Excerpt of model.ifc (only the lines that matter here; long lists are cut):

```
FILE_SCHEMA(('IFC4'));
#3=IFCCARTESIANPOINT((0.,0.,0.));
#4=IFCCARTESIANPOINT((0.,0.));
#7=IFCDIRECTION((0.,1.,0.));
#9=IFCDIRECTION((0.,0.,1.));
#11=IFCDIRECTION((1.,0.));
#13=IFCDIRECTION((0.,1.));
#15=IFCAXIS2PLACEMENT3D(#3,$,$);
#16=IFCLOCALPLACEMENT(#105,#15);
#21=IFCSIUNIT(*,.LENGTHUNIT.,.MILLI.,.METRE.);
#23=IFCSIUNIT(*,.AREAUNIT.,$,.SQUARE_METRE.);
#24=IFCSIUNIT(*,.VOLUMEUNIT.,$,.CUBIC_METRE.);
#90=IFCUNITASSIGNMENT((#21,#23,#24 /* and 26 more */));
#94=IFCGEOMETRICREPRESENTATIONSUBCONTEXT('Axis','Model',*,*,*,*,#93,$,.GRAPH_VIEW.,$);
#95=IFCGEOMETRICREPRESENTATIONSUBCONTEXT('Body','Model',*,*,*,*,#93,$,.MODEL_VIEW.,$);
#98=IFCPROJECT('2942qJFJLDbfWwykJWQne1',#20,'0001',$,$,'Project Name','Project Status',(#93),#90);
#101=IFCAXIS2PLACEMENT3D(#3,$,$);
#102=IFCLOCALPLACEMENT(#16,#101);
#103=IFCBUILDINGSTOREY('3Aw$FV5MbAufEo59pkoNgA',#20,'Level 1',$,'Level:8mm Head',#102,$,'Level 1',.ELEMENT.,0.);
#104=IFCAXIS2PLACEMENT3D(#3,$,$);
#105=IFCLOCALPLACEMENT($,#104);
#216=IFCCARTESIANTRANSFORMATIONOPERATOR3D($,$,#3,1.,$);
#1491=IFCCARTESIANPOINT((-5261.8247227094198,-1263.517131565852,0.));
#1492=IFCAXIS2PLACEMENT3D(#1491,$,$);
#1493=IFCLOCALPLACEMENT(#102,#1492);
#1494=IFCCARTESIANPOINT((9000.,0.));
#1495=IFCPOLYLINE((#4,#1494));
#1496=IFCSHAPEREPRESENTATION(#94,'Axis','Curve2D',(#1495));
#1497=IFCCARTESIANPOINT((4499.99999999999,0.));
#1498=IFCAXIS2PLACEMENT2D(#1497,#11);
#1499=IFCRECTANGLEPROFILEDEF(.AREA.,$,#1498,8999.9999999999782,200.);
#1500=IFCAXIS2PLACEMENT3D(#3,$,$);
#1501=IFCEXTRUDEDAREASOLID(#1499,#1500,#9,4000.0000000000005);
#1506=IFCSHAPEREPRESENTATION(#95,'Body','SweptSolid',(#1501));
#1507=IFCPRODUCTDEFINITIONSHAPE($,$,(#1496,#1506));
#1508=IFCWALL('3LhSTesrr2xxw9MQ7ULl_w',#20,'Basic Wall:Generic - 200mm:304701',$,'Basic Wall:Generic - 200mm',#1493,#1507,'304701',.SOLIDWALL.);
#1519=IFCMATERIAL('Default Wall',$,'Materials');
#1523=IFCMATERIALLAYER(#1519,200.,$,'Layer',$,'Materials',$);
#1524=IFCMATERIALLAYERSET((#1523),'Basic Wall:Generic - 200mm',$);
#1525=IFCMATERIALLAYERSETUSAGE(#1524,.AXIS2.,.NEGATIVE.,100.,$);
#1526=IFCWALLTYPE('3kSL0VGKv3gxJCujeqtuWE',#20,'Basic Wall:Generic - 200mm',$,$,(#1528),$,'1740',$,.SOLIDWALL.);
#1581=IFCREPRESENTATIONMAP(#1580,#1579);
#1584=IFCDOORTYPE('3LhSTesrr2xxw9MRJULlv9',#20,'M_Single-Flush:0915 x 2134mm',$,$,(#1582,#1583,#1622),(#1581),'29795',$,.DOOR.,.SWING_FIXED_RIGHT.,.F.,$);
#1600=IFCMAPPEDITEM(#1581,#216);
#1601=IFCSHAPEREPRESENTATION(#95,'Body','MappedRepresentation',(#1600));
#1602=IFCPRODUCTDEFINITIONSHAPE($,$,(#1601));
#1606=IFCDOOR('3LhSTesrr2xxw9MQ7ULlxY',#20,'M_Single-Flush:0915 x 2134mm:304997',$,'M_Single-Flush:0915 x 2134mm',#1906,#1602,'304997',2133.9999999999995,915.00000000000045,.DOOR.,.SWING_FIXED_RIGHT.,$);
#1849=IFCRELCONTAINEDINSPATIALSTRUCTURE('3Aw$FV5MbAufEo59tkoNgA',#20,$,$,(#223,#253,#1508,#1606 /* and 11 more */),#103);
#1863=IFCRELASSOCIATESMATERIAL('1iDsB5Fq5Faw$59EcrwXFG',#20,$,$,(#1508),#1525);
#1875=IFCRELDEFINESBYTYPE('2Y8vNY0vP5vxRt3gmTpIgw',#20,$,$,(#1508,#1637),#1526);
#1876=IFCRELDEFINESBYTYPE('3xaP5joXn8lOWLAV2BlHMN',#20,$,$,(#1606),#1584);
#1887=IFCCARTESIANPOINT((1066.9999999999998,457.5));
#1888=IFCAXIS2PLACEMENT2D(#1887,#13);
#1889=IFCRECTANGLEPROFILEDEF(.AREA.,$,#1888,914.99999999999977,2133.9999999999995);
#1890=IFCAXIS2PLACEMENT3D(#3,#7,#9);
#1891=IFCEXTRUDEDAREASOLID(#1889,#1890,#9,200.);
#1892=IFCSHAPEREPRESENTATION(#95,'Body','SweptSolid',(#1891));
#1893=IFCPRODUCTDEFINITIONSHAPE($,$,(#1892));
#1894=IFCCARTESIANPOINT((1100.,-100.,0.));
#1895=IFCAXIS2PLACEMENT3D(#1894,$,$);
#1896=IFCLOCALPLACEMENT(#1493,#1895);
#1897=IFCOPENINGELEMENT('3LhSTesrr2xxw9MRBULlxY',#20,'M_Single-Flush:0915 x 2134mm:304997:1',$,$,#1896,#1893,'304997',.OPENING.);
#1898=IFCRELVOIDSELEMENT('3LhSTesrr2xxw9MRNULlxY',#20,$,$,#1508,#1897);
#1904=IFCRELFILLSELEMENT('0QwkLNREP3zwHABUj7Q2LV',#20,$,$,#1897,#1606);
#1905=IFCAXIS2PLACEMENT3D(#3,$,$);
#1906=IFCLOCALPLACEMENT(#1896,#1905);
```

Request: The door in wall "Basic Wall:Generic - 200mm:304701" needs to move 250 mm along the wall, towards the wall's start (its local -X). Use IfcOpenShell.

```python
import ifcopenshell
import ifcopenshell.api.geometry
import ifcopenshell.util.placement

model = ifcopenshell.open("model.ifc")

door = model.by_guid("3LhSTesrr2xxw9MQ7ULlxY")
opening = door.FillsVoids[0].RelatingOpeningElement
wall = opening.VoidsElements[0].RelatingBuildingElement

wall_matrix = ifcopenshell.util.placement.get_local_placement(wall.ObjectPlacement)
shift = wall_matrix[:3, 0] * -250.0
before = ifcopenshell.util.placement.get_local_placement(door.ObjectPlacement)[:3, 3].copy()

# The door is placed relative to its opening, so it follows when the opening moves.
matrix = ifcopenshell.util.placement.get_local_placement(opening.ObjectPlacement)
matrix[:3, 3] += shift
ifcopenshell.api.geometry.edit_object_placement(
    model, product=opening, matrix=matrix, is_si=False, should_transform_children=True
)

after = ifcopenshell.util.placement.get_local_placement(door.ObjectPlacement)[:3, 3]
print("door moved by", (after - before).round(3) + 0.0)

model.write("model_updated.ifc")
```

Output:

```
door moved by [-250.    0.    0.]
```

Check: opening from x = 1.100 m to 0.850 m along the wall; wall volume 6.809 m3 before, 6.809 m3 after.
